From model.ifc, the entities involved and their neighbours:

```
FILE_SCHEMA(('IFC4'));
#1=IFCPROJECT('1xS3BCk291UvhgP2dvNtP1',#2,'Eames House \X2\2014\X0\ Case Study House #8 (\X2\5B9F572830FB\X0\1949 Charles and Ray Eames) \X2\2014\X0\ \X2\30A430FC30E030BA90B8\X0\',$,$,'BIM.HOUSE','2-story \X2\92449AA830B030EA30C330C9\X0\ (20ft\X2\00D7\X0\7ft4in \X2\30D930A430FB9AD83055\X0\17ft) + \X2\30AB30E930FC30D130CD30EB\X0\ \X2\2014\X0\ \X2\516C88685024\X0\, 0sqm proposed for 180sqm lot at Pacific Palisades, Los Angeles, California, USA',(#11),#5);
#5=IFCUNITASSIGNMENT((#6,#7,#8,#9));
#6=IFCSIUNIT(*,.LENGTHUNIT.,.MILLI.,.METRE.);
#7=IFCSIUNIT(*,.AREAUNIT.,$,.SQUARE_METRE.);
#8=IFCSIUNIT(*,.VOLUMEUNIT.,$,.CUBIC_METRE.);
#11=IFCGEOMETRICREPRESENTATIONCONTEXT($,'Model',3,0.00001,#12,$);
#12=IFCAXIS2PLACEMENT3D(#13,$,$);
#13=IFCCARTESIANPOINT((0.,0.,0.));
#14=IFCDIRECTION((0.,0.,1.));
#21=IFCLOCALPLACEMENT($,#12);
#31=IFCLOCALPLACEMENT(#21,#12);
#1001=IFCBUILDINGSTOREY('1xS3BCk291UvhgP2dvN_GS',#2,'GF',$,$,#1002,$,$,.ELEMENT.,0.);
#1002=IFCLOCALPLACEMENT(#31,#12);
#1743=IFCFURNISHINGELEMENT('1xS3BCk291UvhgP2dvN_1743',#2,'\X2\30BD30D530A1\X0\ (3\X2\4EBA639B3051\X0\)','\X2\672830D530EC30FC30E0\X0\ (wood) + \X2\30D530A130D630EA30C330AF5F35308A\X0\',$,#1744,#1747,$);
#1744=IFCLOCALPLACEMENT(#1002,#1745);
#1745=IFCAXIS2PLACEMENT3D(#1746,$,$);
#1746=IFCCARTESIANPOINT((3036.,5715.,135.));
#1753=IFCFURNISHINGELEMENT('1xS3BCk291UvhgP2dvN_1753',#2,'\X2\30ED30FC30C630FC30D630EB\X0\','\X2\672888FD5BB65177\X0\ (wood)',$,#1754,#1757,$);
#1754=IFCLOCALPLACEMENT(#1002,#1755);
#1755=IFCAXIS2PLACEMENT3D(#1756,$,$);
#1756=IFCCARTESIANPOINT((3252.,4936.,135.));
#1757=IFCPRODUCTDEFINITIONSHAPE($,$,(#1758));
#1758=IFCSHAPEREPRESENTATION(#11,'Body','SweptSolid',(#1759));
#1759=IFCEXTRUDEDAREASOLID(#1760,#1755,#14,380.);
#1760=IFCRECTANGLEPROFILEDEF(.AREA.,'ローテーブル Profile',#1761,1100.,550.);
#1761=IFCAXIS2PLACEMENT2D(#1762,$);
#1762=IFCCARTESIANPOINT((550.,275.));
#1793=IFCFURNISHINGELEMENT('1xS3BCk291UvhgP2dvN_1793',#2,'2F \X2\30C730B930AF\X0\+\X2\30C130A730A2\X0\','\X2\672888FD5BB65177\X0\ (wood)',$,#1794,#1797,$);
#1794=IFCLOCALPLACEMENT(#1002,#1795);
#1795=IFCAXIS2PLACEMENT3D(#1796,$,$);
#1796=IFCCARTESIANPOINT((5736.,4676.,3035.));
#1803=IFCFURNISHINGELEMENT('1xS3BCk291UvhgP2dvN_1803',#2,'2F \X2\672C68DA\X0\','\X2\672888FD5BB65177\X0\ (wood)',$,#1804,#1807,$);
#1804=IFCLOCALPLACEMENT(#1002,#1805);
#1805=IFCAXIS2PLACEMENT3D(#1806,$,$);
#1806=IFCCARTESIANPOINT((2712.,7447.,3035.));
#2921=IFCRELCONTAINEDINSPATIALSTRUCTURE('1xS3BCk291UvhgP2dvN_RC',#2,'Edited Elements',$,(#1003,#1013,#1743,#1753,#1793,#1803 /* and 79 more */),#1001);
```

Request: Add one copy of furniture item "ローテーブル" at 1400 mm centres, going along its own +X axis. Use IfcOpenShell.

```python
import ifcopenshell
import ifcopenshell.api.geometry
import ifcopenshell.api.root
import ifcopenshell.util.element
import ifcopenshell.util.placement
import ifcopenshell.util.unit

model = ifcopenshell.open("model.ifc")
unit_scale = ifcopenshell.util.unit.calculate_unit_scale(model)


def reuse_history(source, copy):
    """copy_class also copies each property set's owner history, people and application; keep the originals."""
    for rel in copy.IsDefinedBy:
        if rel.is_a("IfcRelDefinesByProperties") and (history := rel.RelatingPropertyDefinition.OwnerHistory):
            rel.RelatingPropertyDefinition.OwnerHistory = source.OwnerHistory
            ifcopenshell.util.element.remove_deep2(model, history)


source = model.by_guid("1xS3BCk291UvhgP2dvN_1753")
base = ifcopenshell.util.placement.get_local_placement(source.ObjectPlacement)
step = base[:3, 0] * 1.4 / unit_scale

for i in range(1, 2):
    copy = ifcopenshell.api.root.copy_class(model, product=source)
    copy.Representation = ifcopenshell.util.element.copy_deep(
        model, source.Representation, exclude=["IfcGeometricRepresentationContext", "IfcRepresentationMap"]
    )
    reuse_history(source, copy)
    matrix = base.copy()
    matrix[:3, 3] += i * step
    print("added at", matrix[:3, 3].round(3) + 0.0)
    ifcopenshell.api.geometry.edit_object_placement(model, product=copy, matrix=matrix, is_si=False)

model.write("model_v2.ifc")
```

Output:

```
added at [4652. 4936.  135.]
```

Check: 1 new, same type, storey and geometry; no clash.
